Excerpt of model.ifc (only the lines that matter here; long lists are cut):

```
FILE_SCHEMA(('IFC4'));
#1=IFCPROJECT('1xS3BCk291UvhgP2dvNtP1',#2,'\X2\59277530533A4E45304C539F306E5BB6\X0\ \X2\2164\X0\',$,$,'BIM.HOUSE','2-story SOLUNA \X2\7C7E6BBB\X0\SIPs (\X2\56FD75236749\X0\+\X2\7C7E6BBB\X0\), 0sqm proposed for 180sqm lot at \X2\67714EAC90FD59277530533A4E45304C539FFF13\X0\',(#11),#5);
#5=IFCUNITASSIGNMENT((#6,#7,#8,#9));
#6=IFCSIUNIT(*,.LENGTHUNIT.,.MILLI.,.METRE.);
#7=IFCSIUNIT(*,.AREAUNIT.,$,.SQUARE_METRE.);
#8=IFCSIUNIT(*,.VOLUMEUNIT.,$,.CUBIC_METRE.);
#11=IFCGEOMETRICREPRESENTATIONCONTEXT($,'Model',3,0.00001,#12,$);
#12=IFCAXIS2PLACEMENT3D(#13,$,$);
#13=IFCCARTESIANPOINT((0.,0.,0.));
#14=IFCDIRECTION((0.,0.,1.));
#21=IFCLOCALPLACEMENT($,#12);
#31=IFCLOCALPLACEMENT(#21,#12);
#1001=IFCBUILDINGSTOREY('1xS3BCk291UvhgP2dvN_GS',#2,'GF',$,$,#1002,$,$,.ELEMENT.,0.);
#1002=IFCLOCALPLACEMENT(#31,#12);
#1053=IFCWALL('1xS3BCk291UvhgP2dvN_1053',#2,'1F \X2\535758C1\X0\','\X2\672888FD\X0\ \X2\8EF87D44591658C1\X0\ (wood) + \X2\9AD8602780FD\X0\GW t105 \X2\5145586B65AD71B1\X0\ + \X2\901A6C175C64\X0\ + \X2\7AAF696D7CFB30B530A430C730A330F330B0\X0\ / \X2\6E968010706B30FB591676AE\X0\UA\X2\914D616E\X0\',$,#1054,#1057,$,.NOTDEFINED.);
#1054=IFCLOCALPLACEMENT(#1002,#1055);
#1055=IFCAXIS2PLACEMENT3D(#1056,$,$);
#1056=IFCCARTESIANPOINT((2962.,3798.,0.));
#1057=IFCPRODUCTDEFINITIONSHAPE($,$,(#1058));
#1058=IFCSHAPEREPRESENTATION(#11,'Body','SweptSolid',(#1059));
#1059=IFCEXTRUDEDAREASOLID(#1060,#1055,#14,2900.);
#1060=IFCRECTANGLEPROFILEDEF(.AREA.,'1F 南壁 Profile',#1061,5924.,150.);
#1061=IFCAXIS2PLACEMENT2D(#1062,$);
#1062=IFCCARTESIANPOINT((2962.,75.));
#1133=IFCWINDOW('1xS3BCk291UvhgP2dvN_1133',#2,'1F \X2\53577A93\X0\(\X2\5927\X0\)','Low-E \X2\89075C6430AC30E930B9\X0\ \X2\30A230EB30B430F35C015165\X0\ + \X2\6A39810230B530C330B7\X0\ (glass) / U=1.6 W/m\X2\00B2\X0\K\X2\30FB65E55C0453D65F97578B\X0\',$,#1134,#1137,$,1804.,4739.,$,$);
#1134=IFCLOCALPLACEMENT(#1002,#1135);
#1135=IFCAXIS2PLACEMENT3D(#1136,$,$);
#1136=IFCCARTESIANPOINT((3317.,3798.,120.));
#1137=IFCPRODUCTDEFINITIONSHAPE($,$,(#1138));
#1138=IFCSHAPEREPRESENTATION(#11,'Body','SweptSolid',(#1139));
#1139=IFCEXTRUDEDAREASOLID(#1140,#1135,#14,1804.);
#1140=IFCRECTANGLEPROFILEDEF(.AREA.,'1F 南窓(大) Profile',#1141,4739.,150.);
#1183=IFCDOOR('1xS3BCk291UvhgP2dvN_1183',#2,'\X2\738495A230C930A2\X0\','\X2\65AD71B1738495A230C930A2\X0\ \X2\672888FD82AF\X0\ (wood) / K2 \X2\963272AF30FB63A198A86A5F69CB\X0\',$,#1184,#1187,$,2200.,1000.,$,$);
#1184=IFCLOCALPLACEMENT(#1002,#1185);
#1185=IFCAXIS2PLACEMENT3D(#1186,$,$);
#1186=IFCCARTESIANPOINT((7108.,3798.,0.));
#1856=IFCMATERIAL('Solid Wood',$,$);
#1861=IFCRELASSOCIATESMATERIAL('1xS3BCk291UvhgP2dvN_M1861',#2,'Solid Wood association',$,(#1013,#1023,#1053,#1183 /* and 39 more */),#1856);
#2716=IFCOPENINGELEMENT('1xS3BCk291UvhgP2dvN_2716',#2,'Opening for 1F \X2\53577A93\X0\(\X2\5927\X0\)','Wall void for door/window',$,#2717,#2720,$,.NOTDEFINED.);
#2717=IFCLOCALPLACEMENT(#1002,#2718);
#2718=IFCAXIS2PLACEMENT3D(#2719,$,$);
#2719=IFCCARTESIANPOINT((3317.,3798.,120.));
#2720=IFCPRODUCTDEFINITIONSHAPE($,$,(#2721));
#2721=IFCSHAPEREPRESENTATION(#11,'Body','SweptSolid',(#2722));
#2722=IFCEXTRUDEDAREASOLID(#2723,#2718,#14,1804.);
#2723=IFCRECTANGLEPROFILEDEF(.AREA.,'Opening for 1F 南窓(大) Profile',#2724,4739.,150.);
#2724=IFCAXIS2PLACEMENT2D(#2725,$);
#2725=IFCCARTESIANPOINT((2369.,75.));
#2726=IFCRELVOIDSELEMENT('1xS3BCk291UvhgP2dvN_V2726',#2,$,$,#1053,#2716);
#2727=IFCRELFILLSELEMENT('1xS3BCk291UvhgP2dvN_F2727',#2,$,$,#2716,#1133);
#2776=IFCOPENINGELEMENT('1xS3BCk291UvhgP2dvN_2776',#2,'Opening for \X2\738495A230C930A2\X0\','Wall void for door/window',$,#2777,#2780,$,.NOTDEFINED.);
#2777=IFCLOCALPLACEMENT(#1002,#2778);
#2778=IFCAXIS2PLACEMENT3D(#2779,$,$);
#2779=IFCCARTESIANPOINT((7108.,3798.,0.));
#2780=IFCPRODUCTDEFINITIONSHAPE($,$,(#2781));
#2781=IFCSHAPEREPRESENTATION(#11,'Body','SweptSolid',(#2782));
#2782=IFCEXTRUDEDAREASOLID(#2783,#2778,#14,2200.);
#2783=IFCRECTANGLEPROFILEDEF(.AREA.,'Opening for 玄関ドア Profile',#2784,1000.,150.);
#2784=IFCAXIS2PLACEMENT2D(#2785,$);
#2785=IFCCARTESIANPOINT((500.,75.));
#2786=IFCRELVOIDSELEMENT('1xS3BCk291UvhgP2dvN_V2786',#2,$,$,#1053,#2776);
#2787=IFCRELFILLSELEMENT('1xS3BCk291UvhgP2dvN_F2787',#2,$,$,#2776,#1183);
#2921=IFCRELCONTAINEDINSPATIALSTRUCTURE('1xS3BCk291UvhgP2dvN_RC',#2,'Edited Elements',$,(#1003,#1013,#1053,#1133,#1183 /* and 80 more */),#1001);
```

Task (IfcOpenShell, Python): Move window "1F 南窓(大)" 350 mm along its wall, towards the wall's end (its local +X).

```python
import ifcopenshell
import ifcopenshell.api.geometry
import ifcopenshell.util.placement
import ifcopenshell.util.unit

model = ifcopenshell.open("model.ifc")
unit_scale = ifcopenshell.util.unit.calculate_unit_scale(model)

window = model.by_id(1133)
opening = window.FillsVoids[0].RelatingOpeningElement
wall = opening.VoidsElements[0].RelatingBuildingElement

wall_matrix = ifcopenshell.util.placement.get_local_placement(wall.ObjectPlacement)
shift = wall_matrix[:3, 0] * 0.35 / unit_scale
before = ifcopenshell.util.placement.get_local_placement(window.ObjectPlacement)[:3, 3].copy()

# The window is not placed relative to its opening, so move both.
for product in (opening, window):
    matrix = ifcopenshell.util.placement.get_local_placement(product.ObjectPlacement)
    matrix[:3, 3] += shift
    ifcopenshell.api.geometry.edit_object_placement(model, product=product, matrix=matrix, is_si=False)

after = ifcopenshell.util.placement.get_local_placement(window.ObjectPlacement)[:3, 3]
print("window moved by", (after - before).round(3) + 0.0)

model.write("model_rev.ifc")
```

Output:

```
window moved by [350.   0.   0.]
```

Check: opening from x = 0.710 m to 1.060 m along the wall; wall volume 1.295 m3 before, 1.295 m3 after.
